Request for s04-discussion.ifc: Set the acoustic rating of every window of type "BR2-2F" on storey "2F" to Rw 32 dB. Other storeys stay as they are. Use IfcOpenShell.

First a look at what the model holds.

```python
import ifcopenshell
import ifcopenshell.util.element

model = ifcopenshell.open("s04-discussion.ifc")
print(model.schema)
storey = next(s for s in model.by_type("IfcBuildingStorey") if s.Name == "2F")
windows = [e for e in ifcopenshell.util.element.get_decomposition(storey) if e.is_a("IfcWindow")]
seen = {}
for e in windows:
    element_type = ifcopenshell.util.element.get_type(e)
    key = (element_type.Name if element_type != e and element_type else None, ifcopenshell.util.element.get_pset(e, "Pset_WindowCommon", "AcousticRating"))
    seen[key] = seen.get(key, 0) + 1
for (name, value), count in sorted(seen.items(), key=str):
    print(count, "x", name, "|", value)
```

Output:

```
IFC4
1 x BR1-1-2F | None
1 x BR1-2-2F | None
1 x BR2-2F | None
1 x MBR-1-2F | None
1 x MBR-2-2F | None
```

```python
import ifcopenshell
import ifcopenshell.api.pset
import ifcopenshell.util.element

model = ifcopenshell.open("s04-discussion.ifc")

storey = next(s for s in model.by_type("IfcBuildingStorey") if s.Name == "2F")
windows = [e for e in ifcopenshell.util.element.get_decomposition(storey) if e.is_a("IfcWindow")]

count = 0
for e in windows:
    element_type = ifcopenshell.util.element.get_type(e)
    if element_type in (None, e) or element_type.Name != "BR2-2F":
        continue
    # add_pset returns the element's existing set when there is one.
    pset = ifcopenshell.api.pset.add_pset(model, product=e, name="Pset_WindowCommon")
    ifcopenshell.api.pset.edit_pset(model, pset=pset, properties={"AcousticRating": "Rw 32 dB"})
    count += 1

print(count, "windows updated")

model.write("s04-discussion_rev.ifc")
```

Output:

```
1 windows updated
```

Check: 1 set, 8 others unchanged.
